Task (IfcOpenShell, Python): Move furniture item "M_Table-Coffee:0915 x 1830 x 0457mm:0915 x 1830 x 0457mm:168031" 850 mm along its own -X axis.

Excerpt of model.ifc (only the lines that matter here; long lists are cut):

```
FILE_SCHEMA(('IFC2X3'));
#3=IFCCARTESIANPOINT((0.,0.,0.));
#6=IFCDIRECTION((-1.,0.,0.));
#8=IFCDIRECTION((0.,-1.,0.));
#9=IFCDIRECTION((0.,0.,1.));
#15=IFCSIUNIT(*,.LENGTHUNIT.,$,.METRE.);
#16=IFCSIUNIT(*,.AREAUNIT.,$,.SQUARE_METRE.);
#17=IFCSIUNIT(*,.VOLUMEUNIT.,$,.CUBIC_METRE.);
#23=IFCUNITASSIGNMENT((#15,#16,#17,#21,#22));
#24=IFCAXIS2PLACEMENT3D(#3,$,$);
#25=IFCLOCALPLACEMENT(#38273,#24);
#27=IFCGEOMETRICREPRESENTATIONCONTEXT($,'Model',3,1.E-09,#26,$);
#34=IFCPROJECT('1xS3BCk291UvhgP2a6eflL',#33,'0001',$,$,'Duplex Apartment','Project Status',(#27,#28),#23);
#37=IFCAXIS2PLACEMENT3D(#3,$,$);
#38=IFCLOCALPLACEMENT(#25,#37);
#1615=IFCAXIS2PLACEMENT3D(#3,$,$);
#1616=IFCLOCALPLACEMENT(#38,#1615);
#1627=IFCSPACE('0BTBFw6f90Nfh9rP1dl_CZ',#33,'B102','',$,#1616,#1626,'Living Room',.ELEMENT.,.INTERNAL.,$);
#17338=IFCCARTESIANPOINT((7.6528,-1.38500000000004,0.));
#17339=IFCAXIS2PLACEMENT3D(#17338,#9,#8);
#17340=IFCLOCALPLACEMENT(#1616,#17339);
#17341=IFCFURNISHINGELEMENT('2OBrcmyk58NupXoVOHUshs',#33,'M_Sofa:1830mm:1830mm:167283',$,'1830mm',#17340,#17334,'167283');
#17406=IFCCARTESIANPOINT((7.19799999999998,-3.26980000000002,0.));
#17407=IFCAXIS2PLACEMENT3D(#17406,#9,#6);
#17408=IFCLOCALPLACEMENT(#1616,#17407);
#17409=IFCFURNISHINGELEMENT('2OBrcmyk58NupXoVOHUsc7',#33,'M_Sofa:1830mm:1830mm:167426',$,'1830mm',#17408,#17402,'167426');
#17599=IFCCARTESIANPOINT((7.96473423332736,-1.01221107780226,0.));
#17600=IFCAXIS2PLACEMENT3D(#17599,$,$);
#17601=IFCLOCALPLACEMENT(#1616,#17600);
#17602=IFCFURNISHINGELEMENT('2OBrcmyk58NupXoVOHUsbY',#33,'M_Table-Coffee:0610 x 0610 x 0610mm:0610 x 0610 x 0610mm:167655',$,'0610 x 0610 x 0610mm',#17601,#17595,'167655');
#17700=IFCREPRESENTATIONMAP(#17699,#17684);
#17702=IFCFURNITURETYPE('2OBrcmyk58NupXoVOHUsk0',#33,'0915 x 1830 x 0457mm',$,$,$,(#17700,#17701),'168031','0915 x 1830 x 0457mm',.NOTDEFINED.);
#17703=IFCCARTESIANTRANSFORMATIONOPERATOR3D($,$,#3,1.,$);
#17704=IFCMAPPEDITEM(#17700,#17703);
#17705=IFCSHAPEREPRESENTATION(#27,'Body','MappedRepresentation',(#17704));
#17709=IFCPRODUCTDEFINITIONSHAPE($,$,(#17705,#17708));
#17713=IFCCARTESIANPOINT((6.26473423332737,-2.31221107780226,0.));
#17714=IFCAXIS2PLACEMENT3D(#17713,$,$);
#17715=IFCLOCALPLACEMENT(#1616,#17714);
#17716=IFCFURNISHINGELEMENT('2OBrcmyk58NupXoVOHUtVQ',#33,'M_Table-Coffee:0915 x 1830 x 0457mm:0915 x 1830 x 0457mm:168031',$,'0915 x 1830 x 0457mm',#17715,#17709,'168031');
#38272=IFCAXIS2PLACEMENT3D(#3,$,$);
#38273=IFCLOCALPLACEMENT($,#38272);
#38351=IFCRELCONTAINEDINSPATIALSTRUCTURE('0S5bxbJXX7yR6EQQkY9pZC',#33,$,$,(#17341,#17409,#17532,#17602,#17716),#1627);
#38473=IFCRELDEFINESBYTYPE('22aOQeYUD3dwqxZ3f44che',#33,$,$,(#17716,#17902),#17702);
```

```python
import ifcopenshell
import ifcopenshell.api.geometry
import ifcopenshell.util.placement

model = ifcopenshell.open("model.ifc")

item = model.by_guid("2OBrcmyk58NupXoVOHUtVQ")
matrix = ifcopenshell.util.placement.get_local_placement(item.ObjectPlacement)
matrix[:3, 3] -= matrix[:3, 0] * 0.85
ifcopenshell.api.geometry.edit_object_placement(model, product=item, matrix=matrix, is_si=False)

print(ifcopenshell.util.placement.get_local_placement(item.ObjectPlacement).round(3) + 0.0)

model.write("model_edited.ifc")
```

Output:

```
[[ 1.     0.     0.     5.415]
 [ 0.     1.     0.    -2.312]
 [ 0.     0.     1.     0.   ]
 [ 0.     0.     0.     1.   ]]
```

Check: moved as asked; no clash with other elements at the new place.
